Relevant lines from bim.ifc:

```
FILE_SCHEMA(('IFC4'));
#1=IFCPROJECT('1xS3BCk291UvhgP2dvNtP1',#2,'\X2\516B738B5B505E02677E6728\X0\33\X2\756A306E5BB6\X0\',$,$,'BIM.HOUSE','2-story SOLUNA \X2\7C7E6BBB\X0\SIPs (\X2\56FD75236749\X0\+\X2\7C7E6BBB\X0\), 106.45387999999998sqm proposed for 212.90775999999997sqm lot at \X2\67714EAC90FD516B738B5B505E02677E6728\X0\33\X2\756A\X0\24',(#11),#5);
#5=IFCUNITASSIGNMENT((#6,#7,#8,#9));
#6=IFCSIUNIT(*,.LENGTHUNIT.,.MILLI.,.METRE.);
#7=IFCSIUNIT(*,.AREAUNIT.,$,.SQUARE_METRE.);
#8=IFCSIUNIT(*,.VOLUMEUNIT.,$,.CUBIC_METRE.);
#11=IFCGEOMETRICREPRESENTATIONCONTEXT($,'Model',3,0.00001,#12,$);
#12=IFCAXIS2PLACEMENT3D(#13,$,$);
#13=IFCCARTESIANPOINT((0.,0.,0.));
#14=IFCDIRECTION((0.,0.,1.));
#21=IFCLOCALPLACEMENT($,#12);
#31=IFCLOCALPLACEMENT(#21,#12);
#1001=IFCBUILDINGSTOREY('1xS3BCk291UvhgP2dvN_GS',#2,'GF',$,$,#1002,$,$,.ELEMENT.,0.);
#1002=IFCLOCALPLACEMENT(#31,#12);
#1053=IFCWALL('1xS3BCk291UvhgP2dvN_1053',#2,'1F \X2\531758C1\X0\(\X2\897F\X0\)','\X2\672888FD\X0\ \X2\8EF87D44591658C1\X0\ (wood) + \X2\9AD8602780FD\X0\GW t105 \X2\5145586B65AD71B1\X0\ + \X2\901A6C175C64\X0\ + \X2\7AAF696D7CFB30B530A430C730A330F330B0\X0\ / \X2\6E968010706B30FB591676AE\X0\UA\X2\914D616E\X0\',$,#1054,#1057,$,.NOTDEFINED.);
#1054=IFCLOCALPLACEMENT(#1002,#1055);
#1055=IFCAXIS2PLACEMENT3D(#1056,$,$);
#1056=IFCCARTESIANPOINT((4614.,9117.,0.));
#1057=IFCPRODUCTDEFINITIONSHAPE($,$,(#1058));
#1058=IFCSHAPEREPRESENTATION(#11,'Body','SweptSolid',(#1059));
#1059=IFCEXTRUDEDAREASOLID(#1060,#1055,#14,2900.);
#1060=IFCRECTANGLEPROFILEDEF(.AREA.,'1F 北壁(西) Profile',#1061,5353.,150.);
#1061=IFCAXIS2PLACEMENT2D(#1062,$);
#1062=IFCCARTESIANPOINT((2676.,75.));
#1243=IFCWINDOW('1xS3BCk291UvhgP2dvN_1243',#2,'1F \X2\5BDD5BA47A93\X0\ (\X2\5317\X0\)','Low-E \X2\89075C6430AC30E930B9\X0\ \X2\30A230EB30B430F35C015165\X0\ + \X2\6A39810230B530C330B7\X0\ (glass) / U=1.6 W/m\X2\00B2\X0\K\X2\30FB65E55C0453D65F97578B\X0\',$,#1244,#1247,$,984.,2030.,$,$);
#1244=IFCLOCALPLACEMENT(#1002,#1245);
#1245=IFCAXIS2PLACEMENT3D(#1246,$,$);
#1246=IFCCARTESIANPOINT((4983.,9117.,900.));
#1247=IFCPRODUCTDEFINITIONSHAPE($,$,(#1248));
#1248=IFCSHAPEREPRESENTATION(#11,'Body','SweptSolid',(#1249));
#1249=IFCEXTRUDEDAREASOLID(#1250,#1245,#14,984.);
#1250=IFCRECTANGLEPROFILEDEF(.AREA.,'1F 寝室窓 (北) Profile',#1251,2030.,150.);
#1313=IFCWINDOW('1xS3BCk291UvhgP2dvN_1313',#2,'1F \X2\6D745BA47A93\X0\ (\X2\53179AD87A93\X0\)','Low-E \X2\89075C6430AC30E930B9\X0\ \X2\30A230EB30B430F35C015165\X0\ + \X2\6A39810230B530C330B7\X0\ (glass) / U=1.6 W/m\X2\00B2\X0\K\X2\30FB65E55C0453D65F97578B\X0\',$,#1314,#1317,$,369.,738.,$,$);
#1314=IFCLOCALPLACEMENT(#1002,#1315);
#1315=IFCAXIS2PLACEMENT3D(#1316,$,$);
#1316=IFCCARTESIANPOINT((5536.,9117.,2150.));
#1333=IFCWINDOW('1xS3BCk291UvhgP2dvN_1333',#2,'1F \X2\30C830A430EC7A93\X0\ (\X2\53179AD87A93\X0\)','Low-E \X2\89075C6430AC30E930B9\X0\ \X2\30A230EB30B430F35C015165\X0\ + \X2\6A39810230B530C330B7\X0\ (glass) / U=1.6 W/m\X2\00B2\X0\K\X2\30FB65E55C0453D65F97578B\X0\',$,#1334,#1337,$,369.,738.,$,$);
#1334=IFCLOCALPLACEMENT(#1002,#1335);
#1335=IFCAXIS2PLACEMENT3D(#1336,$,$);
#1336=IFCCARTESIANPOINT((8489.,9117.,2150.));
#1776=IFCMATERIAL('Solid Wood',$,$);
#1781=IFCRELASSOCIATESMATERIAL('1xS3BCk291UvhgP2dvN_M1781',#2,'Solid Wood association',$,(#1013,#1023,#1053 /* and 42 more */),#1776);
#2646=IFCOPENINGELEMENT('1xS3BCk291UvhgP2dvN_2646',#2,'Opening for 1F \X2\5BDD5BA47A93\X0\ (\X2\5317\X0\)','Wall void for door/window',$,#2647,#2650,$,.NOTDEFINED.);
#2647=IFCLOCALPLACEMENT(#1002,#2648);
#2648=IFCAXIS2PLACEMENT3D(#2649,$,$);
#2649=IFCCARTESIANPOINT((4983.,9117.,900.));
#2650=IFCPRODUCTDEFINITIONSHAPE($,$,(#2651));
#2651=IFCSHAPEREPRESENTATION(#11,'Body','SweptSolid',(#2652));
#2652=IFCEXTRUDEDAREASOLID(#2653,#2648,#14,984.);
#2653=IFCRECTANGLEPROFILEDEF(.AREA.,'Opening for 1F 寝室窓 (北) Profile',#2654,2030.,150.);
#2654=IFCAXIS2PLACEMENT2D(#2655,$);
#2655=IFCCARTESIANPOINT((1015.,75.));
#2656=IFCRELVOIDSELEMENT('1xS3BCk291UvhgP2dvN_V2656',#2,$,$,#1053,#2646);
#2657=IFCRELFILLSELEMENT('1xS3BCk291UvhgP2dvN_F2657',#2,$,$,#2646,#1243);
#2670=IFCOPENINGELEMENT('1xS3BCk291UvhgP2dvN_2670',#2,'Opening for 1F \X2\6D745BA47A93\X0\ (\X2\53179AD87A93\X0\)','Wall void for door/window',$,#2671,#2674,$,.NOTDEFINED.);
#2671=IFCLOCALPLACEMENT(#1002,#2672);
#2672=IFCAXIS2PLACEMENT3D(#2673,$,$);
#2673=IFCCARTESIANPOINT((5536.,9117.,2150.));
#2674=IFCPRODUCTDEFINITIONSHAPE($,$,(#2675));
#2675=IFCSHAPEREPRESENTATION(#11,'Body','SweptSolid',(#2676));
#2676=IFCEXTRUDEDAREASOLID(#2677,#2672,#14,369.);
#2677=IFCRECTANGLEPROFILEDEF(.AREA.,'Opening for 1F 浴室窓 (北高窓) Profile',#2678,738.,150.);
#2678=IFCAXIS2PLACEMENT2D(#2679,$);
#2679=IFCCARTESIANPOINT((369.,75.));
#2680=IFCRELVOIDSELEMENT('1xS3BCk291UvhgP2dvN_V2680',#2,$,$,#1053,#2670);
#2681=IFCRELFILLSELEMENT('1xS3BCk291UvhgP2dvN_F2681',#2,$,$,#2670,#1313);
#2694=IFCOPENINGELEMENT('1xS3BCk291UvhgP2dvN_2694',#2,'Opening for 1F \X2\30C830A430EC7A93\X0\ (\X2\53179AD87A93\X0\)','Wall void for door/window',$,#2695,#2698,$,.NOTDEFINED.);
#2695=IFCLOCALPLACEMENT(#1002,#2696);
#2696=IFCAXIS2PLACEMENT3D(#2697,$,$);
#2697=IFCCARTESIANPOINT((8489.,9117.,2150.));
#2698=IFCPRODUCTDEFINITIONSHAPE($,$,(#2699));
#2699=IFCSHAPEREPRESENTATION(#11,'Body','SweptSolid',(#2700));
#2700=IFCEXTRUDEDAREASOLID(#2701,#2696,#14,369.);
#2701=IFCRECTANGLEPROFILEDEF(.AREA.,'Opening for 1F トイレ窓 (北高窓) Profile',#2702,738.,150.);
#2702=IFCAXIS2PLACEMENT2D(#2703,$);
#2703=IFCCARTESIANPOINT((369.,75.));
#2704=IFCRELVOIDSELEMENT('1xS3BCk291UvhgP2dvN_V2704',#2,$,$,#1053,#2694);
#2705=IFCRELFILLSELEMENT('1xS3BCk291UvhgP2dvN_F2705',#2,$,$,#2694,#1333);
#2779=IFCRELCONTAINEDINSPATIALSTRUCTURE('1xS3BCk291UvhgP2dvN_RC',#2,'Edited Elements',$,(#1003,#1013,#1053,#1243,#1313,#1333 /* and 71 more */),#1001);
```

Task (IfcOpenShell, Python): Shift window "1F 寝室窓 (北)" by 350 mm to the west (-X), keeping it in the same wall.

```python
import ifcopenshell
import ifcopenshell.api.geometry
import ifcopenshell.util.placement
import ifcopenshell.util.unit

model = ifcopenshell.open("bim.ifc")
unit_scale = ifcopenshell.util.unit.calculate_unit_scale(model)

window = model.by_guid("1xS3BCk291UvhgP2dvN_1243")
opening = window.FillsVoids[0].RelatingOpeningElement
wall = opening.VoidsElements[0].RelatingBuildingElement

wall_matrix = ifcopenshell.util.placement.get_local_placement(wall.ObjectPlacement)
shift = wall_matrix[:3, 0] * -0.35 / unit_scale
before = ifcopenshell.util.placement.get_local_placement(window.ObjectPlacement)[:3, 3].copy()

# The window is not placed relative to its opening, so move both.
for product in (opening, window):
    matrix = ifcopenshell.util.placement.get_local_placement(product.ObjectPlacement)
    matrix[:3, 3] += shift
    ifcopenshell.api.geometry.edit_object_placement(model, product=product, matrix=matrix, is_si=False)

after = ifcopenshell.util.placement.get_local_placement(window.ObjectPlacement)[:3, 3]
print("window moved by", (after - before).round(3) + 0.0)

model.write("bim_v2.ifc")
```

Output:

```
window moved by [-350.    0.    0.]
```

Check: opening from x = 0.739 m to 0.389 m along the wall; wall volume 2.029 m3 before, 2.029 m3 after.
